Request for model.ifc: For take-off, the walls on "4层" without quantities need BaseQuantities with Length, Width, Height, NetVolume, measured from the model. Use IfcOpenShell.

First a look at what the model holds.

```python
import ifcopenshell
import ifcopenshell.util.element
import ifcopenshell.util.unit

model = ifcopenshell.open("model.ifc")
print(model.schema)
for unit_type in ("LENGTHUNIT", "AREAUNIT", "VOLUMEUNIT"):
    print(unit_type, ifcopenshell.util.unit.calculate_unit_scale(model, unit_type))
storey = next(s for s in model.by_type("IfcBuildingStorey") if s.Name == "4层")
walls = [e for e in ifcopenshell.util.element.get_decomposition(storey) if e.is_a("IfcWall")]
for e in sorted(walls, key=lambda e: e.id()):
    print(e.id(), e.is_a(), e.Name, list(ifcopenshell.util.element.get_psets(e, qtos_only=True)), sep=" | ")
```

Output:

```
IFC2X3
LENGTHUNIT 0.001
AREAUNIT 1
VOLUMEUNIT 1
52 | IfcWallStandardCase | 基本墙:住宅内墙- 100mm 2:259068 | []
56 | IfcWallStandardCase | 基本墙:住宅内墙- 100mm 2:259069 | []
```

```python
import ifcopenshell
import ifcopenshell.api.pset
import ifcopenshell.geom
import ifcopenshell.util.element
import ifcopenshell.util.shape
import ifcopenshell.util.unit

model = ifcopenshell.open("model.ifc")
unit_scale = ifcopenshell.util.unit.calculate_unit_scale(model)
volume_scale = ifcopenshell.util.unit.calculate_unit_scale(model, "VOLUMEUNIT")
settings = ifcopenshell.geom.settings()

storey = next(s for s in model.by_type("IfcBuildingStorey") if s.Name == "4层")
walls = [e for e in ifcopenshell.util.element.get_decomposition(storey) if e.is_a("IfcWall")]

for e in sorted(walls, key=lambda e: e.id()):
    if ifcopenshell.util.element.get_psets(e, qtos_only=True, should_inherit=False):
        continue
    # Geometry comes back in metres, in the element's own axes.
    shape = ifcopenshell.geom.create_shape(settings, e)
    values = {
        "Length": ifcopenshell.util.shape.get_x(shape.geometry) / unit_scale,
        "Width": ifcopenshell.util.shape.get_y(shape.geometry) / unit_scale,
        "Height": ifcopenshell.util.shape.get_z(shape.geometry) / unit_scale,
        "NetVolume": ifcopenshell.util.shape.get_volume(shape.geometry) / volume_scale,
    }
    qto = ifcopenshell.api.pset.add_qto(model, product=e, name="BaseQuantities")
    ifcopenshell.api.pset.edit_qto(model, qto=qto, properties=values)
    print(e.id(), {k: round(v, 3) for k, v in values.items()})

model.write("model-out.ifc")
```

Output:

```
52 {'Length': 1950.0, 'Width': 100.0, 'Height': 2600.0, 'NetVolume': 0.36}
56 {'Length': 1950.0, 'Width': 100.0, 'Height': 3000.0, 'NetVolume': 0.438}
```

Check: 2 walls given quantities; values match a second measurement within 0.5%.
